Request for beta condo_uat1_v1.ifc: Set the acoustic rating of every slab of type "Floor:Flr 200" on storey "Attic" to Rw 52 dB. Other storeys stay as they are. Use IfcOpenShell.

First a look at what the model holds.

```python
import ifcopenshell
import ifcopenshell.util.element

model = ifcopenshell.open("beta condo_uat1_v1.ifc")
print(model.schema)
storey = next(s for s in model.by_type("IfcBuildingStorey") if s.Name == "Attic")
slabs = [e for e in ifcopenshell.util.element.get_decomposition(storey) if e.is_a("IfcSlab")]
seen = {}
for e in slabs:
    element_type = ifcopenshell.util.element.get_type(e)
    key = (element_type.Name if element_type != e and element_type else None, ifcopenshell.util.element.get_pset(e, "Pset_SlabCommon", "AcousticRating"))
    seen[key] = seen.get(key, 0) + 1
for (name, value), count in sorted(seen.items(), key=str):
    print(count, "x", name, "|", value)
```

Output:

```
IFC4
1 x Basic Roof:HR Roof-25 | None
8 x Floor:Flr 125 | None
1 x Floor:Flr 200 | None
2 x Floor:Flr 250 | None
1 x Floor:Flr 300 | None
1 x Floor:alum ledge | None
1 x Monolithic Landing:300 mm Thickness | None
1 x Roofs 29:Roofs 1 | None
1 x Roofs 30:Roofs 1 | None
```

```python
import ifcopenshell
import ifcopenshell.api.pset
import ifcopenshell.util.element

model = ifcopenshell.open("beta condo_uat1_v1.ifc")

storey = next(s for s in model.by_type("IfcBuildingStorey") if s.Name == "Attic")
slabs = [e for e in ifcopenshell.util.element.get_decomposition(storey) if e.is_a("IfcSlab")]

count = 0
for e in slabs:
    element_type = ifcopenshell.util.element.get_type(e)
    if element_type in (None, e) or element_type.Name != "Floor:Flr 200":
        continue
    # add_pset returns the element's existing set when there is one.
    pset = ifcopenshell.api.pset.add_pset(model, product=e, name="Pset_SlabCommon")
    ifcopenshell.api.pset.edit_pset(model, pset=pset, properties={"AcousticRating": "Rw 52 dB"})
    count += 1

print(count, "slabs updated")

model.write("beta condo_uat1_v1_rev.ifc")
```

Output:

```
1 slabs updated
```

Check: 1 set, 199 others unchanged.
